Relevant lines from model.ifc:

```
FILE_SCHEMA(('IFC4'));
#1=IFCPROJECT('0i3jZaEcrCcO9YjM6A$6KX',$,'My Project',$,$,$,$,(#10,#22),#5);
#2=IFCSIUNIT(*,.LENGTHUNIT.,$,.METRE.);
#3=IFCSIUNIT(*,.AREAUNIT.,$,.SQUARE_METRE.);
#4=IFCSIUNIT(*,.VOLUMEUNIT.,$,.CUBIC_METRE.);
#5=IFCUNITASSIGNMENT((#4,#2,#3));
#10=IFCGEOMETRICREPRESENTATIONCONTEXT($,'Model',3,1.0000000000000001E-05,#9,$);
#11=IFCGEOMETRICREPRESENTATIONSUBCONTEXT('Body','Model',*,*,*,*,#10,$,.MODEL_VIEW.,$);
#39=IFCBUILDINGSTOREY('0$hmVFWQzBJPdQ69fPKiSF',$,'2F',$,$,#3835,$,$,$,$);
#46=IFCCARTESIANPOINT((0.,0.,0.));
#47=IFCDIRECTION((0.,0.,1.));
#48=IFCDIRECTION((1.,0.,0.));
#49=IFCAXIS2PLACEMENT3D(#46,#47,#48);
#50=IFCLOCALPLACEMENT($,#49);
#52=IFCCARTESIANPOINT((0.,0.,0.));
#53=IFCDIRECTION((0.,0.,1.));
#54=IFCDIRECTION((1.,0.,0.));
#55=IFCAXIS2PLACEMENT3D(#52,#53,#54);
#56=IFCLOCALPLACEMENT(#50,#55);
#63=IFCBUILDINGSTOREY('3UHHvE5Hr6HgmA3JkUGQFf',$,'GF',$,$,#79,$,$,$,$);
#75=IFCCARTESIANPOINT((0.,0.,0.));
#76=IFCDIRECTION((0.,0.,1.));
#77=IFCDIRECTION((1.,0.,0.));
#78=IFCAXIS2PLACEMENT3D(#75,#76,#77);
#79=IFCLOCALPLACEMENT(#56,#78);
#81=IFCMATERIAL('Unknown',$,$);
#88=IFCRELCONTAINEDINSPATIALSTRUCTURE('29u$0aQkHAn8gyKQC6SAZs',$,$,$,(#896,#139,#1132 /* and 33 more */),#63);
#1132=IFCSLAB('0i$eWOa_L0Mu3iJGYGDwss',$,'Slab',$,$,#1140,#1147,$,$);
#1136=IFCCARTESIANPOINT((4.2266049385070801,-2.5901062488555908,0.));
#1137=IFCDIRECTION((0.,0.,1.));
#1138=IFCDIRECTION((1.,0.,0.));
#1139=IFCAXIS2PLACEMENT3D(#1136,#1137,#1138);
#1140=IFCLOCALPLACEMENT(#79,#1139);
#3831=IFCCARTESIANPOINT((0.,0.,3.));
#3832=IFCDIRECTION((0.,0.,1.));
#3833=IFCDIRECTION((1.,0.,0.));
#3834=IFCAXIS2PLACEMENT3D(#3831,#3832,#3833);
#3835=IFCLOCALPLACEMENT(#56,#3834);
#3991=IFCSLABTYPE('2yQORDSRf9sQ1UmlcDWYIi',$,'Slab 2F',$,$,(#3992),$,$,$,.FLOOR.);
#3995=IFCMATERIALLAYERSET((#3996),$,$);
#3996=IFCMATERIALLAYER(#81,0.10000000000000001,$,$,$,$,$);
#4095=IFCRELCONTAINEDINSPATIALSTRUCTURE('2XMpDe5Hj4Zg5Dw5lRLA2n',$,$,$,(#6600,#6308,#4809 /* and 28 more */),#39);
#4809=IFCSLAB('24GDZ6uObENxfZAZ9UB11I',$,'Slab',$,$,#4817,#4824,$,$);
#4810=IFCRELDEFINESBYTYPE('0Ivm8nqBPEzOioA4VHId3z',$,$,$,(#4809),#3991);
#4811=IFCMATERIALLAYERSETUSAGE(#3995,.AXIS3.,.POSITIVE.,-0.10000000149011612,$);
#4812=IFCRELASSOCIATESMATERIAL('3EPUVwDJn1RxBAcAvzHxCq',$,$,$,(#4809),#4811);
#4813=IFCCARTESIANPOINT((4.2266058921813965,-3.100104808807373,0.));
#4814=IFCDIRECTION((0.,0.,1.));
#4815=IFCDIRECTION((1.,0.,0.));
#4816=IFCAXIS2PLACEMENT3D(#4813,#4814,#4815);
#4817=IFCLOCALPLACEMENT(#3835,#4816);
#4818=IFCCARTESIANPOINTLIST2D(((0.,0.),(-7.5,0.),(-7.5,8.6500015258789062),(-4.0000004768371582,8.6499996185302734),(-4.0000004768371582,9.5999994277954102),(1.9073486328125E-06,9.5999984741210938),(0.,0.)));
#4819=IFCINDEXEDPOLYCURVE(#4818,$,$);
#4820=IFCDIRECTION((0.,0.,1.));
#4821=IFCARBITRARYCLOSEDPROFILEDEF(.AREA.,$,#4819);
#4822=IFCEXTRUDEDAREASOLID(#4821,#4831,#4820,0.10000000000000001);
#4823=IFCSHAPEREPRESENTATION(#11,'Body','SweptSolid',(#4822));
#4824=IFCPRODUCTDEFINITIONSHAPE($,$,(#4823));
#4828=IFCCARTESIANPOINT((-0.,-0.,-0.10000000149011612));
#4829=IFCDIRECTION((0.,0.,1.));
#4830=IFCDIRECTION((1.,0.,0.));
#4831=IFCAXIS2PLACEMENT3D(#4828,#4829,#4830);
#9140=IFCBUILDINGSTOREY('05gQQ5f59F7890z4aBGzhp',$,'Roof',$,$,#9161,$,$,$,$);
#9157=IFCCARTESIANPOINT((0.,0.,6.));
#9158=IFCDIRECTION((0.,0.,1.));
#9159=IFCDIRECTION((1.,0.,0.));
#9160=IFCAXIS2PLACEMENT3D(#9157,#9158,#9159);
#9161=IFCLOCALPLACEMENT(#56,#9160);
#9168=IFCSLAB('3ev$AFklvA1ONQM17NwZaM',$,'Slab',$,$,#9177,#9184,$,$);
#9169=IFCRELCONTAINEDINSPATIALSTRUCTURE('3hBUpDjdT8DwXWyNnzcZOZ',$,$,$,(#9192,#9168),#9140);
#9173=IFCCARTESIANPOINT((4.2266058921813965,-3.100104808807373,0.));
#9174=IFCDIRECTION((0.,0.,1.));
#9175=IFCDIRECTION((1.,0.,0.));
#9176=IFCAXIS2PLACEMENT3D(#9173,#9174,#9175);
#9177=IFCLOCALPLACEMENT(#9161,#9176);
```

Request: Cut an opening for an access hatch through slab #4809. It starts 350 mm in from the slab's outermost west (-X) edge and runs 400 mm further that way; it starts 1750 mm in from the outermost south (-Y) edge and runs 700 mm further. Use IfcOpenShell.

```python
import numpy as np
import ifcopenshell
import ifcopenshell.api.feature
import ifcopenshell.api.geometry
import ifcopenshell.api.root
import ifcopenshell.geom
import ifcopenshell.util.placement
import ifcopenshell.util.representation
import ifcopenshell.util.shape
import ifcopenshell.util.unit

model = ifcopenshell.open("model.ifc")
unit_scale = ifcopenshell.util.unit.calculate_unit_scale(model)
settings = ifcopenshell.geom.settings()


def volume(element):
    """Net volume in cubic metres, openings subtracted."""
    shape = ifcopenshell.geom.create_shape(settings, element)
    return ifcopenshell.util.shape.get_volume(shape.geometry)


slab = model.by_guid("24GDZ6uObENxfZAZ9UB11I")
before = volume(slab)

# Extent in the slab's own axes, in metres. The edges named are its -X and -Y sides.
slab_shape = ifcopenshell.geom.create_shape(settings, slab)
vertices = ifcopenshell.util.shape.get_vertices(slab_shape.geometry)
x_min, y_min, bottom = vertices.min(axis=0)
top = vertices[:, 2].max()

opening = ifcopenshell.api.root.create_entity(model, ifc_class="IfcOpeningElement", name="Access hatch opening", predefined_type="OPENING")
context = ifcopenshell.util.representation.get_context(model, "Model", "Body", "MODEL_VIEW")
width, depth = 0.4, 0.7
outline = [(0.0, 0.0), (width, 0.0), (width, depth), (0.0, depth), (0.0, 0.0)]
# Overshoot both faces by 50 mm so the cut is clean.
shape = ifcopenshell.api.geometry.add_slab_representation(
    model, context=context, depth=top - bottom + 0.1, polyline=outline
)
ifcopenshell.api.geometry.assign_representation(model, product=opening, representation=shape)

matrix = ifcopenshell.util.placement.get_local_placement(slab.ObjectPlacement)
matrix[:, 3] = matrix @ np.append(np.array([x_min + 0.35, y_min + 1.75, bottom - 0.05]) / unit_scale, 1.0)
ifcopenshell.api.geometry.edit_object_placement(model, product=opening, matrix=matrix, is_si=False)
ifcopenshell.api.feature.add_feature(model, feature=opening, element=slab)

after = volume(slab)

print(f"slab volume {before:.3f} -> {after:.3f} m3")

model.write("model_updated.ifc")
```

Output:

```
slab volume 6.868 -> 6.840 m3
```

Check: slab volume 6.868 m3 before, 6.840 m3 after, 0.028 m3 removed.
